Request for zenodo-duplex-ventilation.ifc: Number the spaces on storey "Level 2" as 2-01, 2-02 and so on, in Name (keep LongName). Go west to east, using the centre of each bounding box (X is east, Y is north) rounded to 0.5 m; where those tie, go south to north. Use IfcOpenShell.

First a look at what the model holds.

```python
import ifcopenshell
import ifcopenshell.util.element
import ifcopenshell.util.placement

model = ifcopenshell.open("zenodo-duplex-ventilation.ifc")
print(model.schema)
storey = next(s for s in model.by_type("IfcBuildingStorey") if s.Name == "Level 2")
spaces = [e for e in ifcopenshell.util.element.get_decomposition(storey) if e.is_a("IfcSpace")]
for e in sorted(spaces, key=lambda e: e.id()):
    origin = ifcopenshell.util.placement.get_local_placement(e.ObjectPlacement)[:3, 3]
    print(e.id(), e.Name, e.LongName, origin.round(2) + 0.0, sep=" | ")
```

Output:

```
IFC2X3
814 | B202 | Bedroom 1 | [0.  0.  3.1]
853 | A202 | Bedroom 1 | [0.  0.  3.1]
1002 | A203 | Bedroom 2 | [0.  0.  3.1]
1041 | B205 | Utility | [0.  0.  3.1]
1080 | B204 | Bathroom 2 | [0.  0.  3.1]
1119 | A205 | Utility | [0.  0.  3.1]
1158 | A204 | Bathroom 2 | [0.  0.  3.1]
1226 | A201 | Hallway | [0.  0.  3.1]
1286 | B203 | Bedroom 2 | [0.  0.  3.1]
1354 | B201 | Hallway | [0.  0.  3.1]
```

```python
import ifcopenshell
import ifcopenshell.geom
import ifcopenshell.util.element
import ifcopenshell.util.shape

model = ifcopenshell.open("zenodo-duplex-ventilation.ifc")
settings = ifcopenshell.geom.settings()
settings.set("use-world-coords", True)


def centre(element):
    shape = ifcopenshell.geom.create_shape(settings, element)
    return ifcopenshell.util.shape.get_bbox_centroid(shape.geometry)


storey = next(s for s in model.by_type("IfcBuildingStorey") if s.Name == "Level 2")
spaces = [e for e in ifcopenshell.util.element.get_decomposition(storey) if e.is_a("IfcSpace")]

# Insertion points can sit at a corner or the storey origin, so sort by the geometry (in metres).
centres = {e: centre(e) for e in spaces}
spaces.sort(key=lambda e: (round(centres[e][0] / 0.5), centres[e][1]))

for i, e in enumerate(spaces, start=1):
    number = f"2-{i:02d}"
    e.Name = number
    print(e.id(), number)

model.write("zenodo-duplex-ventilation_v2.ifc")
```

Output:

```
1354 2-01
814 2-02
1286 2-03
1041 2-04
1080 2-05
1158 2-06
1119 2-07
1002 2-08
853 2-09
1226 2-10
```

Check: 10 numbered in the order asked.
